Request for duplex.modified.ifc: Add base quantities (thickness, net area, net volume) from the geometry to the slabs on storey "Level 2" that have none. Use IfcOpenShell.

First a look at what the model holds.

```python
import ifcopenshell
import ifcopenshell.util.element
import ifcopenshell.util.unit

model = ifcopenshell.open("duplex.modified.ifc")
print(model.schema)
for unit_type in ("LENGTHUNIT", "AREAUNIT", "VOLUMEUNIT"):
    print(unit_type, ifcopenshell.util.unit.calculate_unit_scale(model, unit_type))
storey = next(s for s in model.by_type("IfcBuildingStorey") if s.Name == "Level 2")
slabs = [e for e in ifcopenshell.util.element.get_decomposition(storey) if e.is_a("IfcSlab")]
for e in sorted(slabs, key=lambda e: e.id()):
    print(e.id(), e.is_a(), e.Name, list(ifcopenshell.util.element.get_psets(e, qtos_only=True)), sep=" | ")
```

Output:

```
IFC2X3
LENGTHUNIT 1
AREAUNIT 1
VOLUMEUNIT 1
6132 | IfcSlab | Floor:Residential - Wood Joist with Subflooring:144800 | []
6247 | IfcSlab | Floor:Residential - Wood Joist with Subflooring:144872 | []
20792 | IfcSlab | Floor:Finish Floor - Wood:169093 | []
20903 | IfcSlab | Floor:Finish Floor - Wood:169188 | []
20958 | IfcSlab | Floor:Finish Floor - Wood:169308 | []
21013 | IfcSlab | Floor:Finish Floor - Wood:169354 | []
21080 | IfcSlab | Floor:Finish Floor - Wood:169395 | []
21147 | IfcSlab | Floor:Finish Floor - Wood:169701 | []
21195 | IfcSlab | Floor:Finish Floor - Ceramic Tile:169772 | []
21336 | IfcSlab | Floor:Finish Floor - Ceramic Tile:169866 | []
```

```python
import ifcopenshell
import ifcopenshell.api.pset
import ifcopenshell.geom
import ifcopenshell.util.element
import ifcopenshell.util.shape
import ifcopenshell.util.unit

model = ifcopenshell.open("duplex.modified.ifc")
unit_scale = ifcopenshell.util.unit.calculate_unit_scale(model)
area_scale = ifcopenshell.util.unit.calculate_unit_scale(model, "AREAUNIT")
volume_scale = ifcopenshell.util.unit.calculate_unit_scale(model, "VOLUMEUNIT")
settings = ifcopenshell.geom.settings()

storey = next(s for s in model.by_type("IfcBuildingStorey") if s.Name == "Level 2")
slabs = [e for e in ifcopenshell.util.element.get_decomposition(storey) if e.is_a("IfcSlab")]

for e in sorted(slabs, key=lambda e: e.id()):
    if ifcopenshell.util.element.get_psets(e, qtos_only=True, should_inherit=False):
        continue
    # Geometry comes back in metres, in the element's own axes.
    shape = ifcopenshell.geom.create_shape(settings, e)
    values = {
        "Width": ifcopenshell.util.shape.get_z(shape.geometry) / unit_scale,
        "NetArea": ifcopenshell.util.shape.get_footprint_area(shape.geometry) / area_scale,
        "NetVolume": ifcopenshell.util.shape.get_volume(shape.geometry) / volume_scale,
    }
    qto = ifcopenshell.api.pset.add_qto(model, product=e, name="BaseQuantities")
    ifcopenshell.api.pset.edit_qto(model, qto=qto, properties=values)
    print(e.id(), {k: round(v, 3) for k, v in values.items()})

model.write("duplex.modified_edited.ifc")
```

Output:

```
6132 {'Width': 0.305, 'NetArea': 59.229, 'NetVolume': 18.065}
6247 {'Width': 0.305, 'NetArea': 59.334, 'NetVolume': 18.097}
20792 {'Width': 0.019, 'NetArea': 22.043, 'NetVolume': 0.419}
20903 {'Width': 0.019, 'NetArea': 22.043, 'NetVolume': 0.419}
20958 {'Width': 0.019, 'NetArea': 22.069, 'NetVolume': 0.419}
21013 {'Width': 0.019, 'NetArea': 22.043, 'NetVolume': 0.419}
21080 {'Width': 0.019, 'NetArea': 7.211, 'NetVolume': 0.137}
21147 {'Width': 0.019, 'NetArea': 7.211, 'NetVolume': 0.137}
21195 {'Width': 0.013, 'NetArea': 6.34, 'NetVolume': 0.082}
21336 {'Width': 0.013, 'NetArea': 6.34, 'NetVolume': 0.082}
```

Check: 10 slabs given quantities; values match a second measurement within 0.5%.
